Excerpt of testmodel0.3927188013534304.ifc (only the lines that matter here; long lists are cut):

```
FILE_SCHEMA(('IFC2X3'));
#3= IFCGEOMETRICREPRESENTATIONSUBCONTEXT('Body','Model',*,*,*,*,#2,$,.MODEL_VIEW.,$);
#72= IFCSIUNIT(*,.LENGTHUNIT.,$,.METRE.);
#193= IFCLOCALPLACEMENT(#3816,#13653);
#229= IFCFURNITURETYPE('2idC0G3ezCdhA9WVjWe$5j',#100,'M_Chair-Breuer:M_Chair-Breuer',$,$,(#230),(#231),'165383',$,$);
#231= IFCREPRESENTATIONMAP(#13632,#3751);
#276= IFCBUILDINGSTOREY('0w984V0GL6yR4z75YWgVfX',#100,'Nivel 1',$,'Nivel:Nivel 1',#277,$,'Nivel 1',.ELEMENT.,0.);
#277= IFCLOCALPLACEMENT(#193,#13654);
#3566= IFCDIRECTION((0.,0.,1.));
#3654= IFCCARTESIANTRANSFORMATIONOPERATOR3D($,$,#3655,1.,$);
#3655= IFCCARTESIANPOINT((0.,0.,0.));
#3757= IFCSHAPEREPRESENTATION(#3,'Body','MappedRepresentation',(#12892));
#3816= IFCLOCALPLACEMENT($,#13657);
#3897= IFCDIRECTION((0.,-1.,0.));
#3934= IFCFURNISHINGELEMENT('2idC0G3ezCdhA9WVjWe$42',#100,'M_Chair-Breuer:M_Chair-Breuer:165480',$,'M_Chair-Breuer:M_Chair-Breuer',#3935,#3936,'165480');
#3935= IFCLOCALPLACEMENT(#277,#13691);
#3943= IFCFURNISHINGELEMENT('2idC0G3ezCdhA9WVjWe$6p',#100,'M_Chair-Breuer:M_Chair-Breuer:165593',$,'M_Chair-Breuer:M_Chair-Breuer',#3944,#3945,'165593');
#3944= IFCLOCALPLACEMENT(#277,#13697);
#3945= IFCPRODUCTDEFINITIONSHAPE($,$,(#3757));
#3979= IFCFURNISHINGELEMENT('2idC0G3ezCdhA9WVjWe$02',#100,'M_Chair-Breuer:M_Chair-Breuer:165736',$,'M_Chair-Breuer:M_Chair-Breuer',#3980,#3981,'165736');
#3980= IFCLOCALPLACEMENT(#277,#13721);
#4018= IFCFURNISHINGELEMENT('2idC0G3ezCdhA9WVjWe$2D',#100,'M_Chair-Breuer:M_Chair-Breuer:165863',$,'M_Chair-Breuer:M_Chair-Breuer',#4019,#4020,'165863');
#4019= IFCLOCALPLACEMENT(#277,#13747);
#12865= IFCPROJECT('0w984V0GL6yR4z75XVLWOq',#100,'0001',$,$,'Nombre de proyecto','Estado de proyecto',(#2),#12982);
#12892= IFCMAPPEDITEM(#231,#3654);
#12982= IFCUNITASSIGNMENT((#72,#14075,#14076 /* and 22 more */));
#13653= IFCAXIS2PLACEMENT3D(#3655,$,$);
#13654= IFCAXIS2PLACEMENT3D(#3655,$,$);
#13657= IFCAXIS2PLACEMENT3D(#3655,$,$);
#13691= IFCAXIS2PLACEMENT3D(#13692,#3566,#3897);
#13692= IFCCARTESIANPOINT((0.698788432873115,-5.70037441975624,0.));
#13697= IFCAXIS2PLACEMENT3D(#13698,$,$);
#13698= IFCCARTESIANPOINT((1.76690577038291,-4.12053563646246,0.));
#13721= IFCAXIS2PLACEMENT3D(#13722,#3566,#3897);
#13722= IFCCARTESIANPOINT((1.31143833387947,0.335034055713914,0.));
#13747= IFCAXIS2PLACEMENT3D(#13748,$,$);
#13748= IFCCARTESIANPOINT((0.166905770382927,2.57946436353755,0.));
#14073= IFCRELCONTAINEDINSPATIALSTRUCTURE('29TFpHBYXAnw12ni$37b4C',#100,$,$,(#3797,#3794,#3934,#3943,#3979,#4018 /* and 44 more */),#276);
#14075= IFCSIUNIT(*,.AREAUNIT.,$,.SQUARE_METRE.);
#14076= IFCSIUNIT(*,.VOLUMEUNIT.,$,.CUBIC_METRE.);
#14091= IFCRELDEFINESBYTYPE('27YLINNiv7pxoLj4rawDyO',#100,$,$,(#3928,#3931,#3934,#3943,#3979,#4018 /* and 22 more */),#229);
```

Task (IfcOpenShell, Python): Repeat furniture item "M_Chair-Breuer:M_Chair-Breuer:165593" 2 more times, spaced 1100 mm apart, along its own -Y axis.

```python
import ifcopenshell
import ifcopenshell.api.geometry
import ifcopenshell.api.root
import ifcopenshell.util.element
import ifcopenshell.util.placement

model = ifcopenshell.open("testmodel0.3927188013534304.ifc")


def reuse_history(source, copy):
    """copy_class also copies each property set's owner history, people and application; keep the originals."""
    for rel in copy.IsDefinedBy:
        if rel.is_a("IfcRelDefinesByProperties") and (history := rel.RelatingPropertyDefinition.OwnerHistory):
            rel.RelatingPropertyDefinition.OwnerHistory = source.OwnerHistory
            ifcopenshell.util.element.remove_deep2(model, history)


source = model.by_guid("2idC0G3ezCdhA9WVjWe$6p")
base = ifcopenshell.util.placement.get_local_placement(source.ObjectPlacement)
step = -base[:3, 1] * 1.1

for i in range(1, 3):
    copy = ifcopenshell.api.root.copy_class(model, product=source)
    copy.Representation = ifcopenshell.util.element.copy_deep(
        model, source.Representation, exclude=["IfcGeometricRepresentationContext", "IfcRepresentationMap"]
    )
    copy.Name = "M_Chair-Breuer:M_Chair-Breuer"
    copy.Tag = None
    reuse_history(source, copy)
    matrix = base.copy()
    matrix[:3, 3] += i * step
    print("added at", matrix[:3, 3].round(3) + 0.0)
    ifcopenshell.api.geometry.edit_object_placement(model, product=copy, matrix=matrix, is_si=False)

model.write("testmodel0.3927188013534304_rev.ifc")
```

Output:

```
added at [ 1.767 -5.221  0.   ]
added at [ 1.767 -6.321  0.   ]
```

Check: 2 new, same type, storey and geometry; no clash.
